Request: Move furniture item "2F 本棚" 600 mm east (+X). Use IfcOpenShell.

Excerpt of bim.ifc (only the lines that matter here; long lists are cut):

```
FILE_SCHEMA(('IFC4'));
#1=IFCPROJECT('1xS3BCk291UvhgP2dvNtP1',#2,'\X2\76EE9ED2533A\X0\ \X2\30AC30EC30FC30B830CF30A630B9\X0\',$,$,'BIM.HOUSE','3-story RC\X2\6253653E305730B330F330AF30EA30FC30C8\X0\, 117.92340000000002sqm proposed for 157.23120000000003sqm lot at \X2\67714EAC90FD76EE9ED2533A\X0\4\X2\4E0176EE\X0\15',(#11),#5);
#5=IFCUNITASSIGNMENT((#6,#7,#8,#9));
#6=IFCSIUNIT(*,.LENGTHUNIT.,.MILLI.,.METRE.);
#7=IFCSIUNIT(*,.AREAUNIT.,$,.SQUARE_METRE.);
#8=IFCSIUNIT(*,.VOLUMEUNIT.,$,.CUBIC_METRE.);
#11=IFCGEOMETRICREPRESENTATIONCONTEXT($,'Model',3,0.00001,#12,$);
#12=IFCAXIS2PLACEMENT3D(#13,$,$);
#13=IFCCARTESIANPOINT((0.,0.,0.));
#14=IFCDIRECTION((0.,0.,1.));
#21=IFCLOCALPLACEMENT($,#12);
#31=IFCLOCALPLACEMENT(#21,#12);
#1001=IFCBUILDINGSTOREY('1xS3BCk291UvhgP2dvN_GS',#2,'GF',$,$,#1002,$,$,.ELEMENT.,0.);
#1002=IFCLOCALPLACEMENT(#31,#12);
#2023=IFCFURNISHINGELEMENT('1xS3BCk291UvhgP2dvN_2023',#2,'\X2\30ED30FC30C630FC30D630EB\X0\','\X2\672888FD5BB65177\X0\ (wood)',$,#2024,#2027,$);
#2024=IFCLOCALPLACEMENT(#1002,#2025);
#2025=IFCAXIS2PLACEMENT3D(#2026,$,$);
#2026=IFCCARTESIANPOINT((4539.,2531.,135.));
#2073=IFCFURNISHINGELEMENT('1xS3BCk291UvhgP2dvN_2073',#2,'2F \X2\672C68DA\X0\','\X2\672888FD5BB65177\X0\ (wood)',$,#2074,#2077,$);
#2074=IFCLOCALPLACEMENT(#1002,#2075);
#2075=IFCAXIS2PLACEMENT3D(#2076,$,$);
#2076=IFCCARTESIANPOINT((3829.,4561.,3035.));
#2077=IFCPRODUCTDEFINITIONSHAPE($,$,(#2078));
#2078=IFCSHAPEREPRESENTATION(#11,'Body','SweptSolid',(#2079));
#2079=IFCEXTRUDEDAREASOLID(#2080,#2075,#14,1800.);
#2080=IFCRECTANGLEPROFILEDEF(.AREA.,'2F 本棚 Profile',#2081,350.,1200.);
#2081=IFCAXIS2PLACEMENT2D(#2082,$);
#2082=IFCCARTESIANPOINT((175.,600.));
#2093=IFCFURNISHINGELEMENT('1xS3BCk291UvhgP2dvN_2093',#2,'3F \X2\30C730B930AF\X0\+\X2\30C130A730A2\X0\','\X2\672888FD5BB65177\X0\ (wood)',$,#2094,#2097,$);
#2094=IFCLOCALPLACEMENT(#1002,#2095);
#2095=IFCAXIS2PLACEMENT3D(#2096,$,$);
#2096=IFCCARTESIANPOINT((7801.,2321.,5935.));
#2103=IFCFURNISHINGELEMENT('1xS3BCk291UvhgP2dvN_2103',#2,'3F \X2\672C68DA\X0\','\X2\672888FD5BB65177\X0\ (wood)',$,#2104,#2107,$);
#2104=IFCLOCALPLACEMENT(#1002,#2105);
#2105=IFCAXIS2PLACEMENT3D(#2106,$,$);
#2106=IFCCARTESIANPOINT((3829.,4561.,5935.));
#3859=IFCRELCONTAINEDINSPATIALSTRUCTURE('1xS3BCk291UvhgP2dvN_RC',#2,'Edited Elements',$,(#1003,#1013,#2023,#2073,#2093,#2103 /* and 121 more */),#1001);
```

```python
import ifcopenshell
import ifcopenshell.api.geometry
import ifcopenshell.util.placement

model = ifcopenshell.open("bim.ifc")

item = model.by_id(2073)
matrix = ifcopenshell.util.placement.get_local_placement(item.ObjectPlacement)
matrix[0, 3] += 600.0
ifcopenshell.api.geometry.edit_object_placement(model, product=item, matrix=matrix, is_si=False)

print(ifcopenshell.util.placement.get_local_placement(item.ObjectPlacement).round(3) + 0.0)

model.write("bim_edited.ifc")
```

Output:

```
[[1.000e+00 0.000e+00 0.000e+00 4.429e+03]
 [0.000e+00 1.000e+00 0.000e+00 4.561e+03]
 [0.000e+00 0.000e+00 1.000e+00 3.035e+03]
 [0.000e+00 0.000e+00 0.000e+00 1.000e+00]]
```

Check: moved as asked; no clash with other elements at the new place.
